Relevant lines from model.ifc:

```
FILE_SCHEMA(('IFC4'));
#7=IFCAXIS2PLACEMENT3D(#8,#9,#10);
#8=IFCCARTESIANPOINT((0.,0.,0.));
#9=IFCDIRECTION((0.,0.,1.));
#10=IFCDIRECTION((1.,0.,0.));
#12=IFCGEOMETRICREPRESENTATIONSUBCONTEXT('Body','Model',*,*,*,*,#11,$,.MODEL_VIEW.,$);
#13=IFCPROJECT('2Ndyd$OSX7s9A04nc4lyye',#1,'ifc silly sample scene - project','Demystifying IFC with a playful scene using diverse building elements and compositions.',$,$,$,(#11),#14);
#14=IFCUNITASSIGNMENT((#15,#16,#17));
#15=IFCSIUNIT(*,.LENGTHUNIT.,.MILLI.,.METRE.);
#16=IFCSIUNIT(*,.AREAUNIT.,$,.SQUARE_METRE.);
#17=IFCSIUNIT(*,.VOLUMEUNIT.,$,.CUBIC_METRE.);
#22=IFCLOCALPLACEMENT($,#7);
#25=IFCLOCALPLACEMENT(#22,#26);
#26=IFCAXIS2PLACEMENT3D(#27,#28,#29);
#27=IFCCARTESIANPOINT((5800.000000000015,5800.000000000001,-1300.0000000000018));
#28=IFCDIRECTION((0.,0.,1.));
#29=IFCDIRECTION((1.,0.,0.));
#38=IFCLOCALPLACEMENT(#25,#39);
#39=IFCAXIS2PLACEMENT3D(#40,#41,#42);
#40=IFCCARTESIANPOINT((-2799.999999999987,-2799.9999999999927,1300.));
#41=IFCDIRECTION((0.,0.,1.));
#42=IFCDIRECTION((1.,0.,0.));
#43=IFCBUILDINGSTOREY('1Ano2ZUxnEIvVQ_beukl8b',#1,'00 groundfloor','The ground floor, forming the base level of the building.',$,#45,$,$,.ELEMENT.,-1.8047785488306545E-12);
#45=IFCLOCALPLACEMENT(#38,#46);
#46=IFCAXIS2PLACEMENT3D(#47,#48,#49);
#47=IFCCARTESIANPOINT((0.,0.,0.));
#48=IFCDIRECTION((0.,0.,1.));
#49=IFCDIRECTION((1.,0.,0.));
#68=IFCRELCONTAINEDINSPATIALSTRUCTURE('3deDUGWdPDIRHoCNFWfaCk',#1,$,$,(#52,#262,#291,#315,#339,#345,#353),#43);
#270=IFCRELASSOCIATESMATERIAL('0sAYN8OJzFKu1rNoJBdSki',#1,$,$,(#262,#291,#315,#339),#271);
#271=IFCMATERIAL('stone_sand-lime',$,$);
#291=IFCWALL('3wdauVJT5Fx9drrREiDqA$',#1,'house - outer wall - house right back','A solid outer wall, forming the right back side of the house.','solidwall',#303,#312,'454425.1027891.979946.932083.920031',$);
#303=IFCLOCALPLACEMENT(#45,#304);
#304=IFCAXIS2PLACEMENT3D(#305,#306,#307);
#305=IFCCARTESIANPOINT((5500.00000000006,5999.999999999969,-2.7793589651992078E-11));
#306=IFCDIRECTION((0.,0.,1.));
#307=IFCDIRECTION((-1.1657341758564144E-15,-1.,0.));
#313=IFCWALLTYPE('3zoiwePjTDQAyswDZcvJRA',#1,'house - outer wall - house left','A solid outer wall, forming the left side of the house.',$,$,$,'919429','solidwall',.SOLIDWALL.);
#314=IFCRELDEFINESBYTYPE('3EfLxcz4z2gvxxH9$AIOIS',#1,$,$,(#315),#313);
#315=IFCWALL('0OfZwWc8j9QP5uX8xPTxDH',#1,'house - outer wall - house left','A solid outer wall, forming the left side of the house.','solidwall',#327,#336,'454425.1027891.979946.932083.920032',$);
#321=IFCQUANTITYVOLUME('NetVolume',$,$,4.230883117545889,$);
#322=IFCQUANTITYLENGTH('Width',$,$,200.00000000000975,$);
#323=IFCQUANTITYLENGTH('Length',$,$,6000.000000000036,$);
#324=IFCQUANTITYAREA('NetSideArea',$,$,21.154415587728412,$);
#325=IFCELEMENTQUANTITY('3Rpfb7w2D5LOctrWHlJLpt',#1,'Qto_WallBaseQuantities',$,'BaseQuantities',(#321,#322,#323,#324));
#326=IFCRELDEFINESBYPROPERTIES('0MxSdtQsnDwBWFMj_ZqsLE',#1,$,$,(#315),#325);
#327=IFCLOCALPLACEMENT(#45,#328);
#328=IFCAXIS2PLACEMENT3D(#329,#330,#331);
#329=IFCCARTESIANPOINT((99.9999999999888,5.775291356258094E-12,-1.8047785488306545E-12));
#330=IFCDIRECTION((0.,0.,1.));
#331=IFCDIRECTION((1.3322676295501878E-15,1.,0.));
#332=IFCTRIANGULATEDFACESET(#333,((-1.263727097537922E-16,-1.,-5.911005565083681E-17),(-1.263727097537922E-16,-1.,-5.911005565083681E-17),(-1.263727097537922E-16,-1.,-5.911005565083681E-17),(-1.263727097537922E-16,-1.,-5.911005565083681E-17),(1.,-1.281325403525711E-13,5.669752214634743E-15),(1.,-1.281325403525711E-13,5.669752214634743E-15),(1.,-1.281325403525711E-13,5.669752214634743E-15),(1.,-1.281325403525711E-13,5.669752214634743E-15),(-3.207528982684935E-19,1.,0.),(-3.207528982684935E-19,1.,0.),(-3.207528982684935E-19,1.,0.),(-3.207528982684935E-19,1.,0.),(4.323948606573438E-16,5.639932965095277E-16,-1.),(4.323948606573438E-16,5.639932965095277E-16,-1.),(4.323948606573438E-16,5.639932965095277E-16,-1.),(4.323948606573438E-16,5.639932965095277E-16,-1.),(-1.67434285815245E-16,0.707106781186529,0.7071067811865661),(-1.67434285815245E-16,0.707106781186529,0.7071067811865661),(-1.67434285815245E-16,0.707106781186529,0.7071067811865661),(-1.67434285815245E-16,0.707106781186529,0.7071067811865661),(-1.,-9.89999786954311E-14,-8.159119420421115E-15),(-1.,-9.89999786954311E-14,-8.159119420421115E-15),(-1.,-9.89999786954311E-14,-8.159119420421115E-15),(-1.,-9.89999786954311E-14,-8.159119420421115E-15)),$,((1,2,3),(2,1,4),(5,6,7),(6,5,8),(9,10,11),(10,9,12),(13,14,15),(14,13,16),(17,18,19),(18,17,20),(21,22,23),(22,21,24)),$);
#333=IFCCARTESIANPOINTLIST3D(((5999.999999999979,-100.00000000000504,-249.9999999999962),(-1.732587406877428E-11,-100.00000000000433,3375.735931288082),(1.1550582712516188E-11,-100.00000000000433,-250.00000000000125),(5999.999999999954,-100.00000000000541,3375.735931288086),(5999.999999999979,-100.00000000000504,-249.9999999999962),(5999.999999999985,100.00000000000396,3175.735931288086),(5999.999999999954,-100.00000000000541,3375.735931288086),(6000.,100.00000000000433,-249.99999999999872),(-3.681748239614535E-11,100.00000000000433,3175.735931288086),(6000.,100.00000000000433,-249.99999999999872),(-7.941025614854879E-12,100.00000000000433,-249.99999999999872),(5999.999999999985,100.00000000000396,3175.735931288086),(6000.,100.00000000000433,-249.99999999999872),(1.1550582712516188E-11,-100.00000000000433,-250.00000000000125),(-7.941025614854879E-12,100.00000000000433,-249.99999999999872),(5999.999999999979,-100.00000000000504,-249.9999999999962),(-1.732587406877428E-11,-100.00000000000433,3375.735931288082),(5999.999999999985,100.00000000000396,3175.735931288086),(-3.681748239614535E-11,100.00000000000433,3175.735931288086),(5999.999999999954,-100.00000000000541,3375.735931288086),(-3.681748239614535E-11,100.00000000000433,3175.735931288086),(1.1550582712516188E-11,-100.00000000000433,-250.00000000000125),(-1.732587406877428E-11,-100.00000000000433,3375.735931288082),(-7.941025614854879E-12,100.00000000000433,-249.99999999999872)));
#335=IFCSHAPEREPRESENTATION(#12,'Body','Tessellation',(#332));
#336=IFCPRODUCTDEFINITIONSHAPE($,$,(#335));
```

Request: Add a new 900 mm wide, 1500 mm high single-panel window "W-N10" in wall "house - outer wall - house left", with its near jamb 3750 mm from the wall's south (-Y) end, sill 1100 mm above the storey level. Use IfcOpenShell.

```python
import numpy as np
import ifcopenshell
import ifcopenshell.api.feature
import ifcopenshell.api.geometry
import ifcopenshell.api.pset
import ifcopenshell.api.root
import ifcopenshell.api.spatial
import ifcopenshell.geom
import ifcopenshell.util.element
import ifcopenshell.util.placement
import ifcopenshell.util.representation
import ifcopenshell.util.shape
import ifcopenshell.util.unit

model = ifcopenshell.open("model.ifc")
unit_scale = ifcopenshell.util.unit.calculate_unit_scale(model)
area_scale = ifcopenshell.util.unit.calculate_unit_scale(model, "AREAUNIT")
volume_scale = ifcopenshell.util.unit.calculate_unit_scale(model, "VOLUMEUNIT")
settings = ifcopenshell.geom.settings()


def volume(element):
    """Net volume in cubic metres, openings subtracted."""
    shape = ifcopenshell.geom.create_shape(settings, element)
    return ifcopenshell.util.shape.get_volume(shape.geometry)


wall = model.by_guid("0OfZwWc8j9QP5uX8xPTxDH")
storey = ifcopenshell.util.element.get_container(wall, ifc_class="IfcBuildingStorey")
context = ifcopenshell.util.representation.get_context(model, "Model", "Body", "MODEL_VIEW")
before = volume(wall)

width, height, from_end, sill = 0.9, 1.5, 3.75, 1.1  # metres

# The wall runs along its own X axis, and the end named is its -X end.
wall_shape = ifcopenshell.geom.create_shape(settings, wall)
x, y, z = ifcopenshell.util.shape.get_vertices(wall_shape.geometry).T
start = x.min() + from_end
face, thickness = float(y.min()), float(y.max() - y.min())
wall_matrix = ifcopenshell.util.placement.get_local_placement(wall.ObjectPlacement)
level = ifcopenshell.util.placement.get_local_placement(storey.ObjectPlacement)[2, 3]


def in_wall(x, y):
    """Placement at x, y metres in the wall's axes, at sill height."""
    matrix = wall_matrix.copy()
    matrix[:, 3] = wall_matrix @ np.array([x / unit_scale, y / unit_scale, 0.0, 1.0])
    matrix[2, 3] = level + sill / unit_scale
    return matrix


# Opening: a box that overshoots both wall faces by 50 mm.
opening = ifcopenshell.api.root.create_entity(model, ifc_class="IfcOpeningElement", predefined_type="OPENING")
box = ifcopenshell.api.geometry.add_wall_representation(
    model, context=context, length=width, height=height, thickness=thickness + 0.1
)
ifcopenshell.api.geometry.assign_representation(model, product=opening, representation=box)
ifcopenshell.api.geometry.edit_object_placement(model, product=opening, matrix=in_wall(start, face - 0.05), is_si=False)
ifcopenshell.api.feature.add_feature(model, feature=opening, element=wall)

window = ifcopenshell.api.root.create_entity(model, ifc_class="IfcWindow", name="W-N10", predefined_type="WINDOW")
window.OverallWidth, window.OverallHeight = width / unit_scale, height / unit_scale
window.PartitioningType = "SINGLE_PANEL"
body = ifcopenshell.api.geometry.add_window_representation(
    model,
    context=context,
    overall_width=window.OverallWidth,
    overall_height=window.OverallHeight,
    partition_type="SINGLE_PANEL",
)
ifcopenshell.api.geometry.assign_representation(model, product=window, representation=body)
ifcopenshell.api.spatial.assign_container(model, products=[window], relating_structure=storey)
ifcopenshell.api.feature.add_filling(model, opening=opening, element=window)

# Centre the window in the wall's thickness.
ifcopenshell.api.geometry.edit_object_placement(model, product=window, matrix=in_wall(start, face), is_si=False)
window_shape = ifcopenshell.geom.create_shape(settings, window)
depth = ifcopenshell.util.shape.get_vertices(window_shape.geometry)[:, 1]
offset = face + thickness / 2 - (depth.min() + depth.max()) / 2
ifcopenshell.api.geometry.edit_object_placement(model, product=window, matrix=in_wall(start, offset), is_si=False)

after = volume(wall)

# Update the wall's stored quantities.
qto = model.by_id(ifcopenshell.util.element.get_pset(wall, "Qto_WallBaseQuantities", should_inherit=False)["id"])
ifcopenshell.api.pset.edit_qto(model, qto=qto, properties={
    "NetVolume": after / volume_scale,
    "NetSideArea": after / thickness / area_scale,
})

print(f"wall volume {before:.3f} -> {after:.3f} m3")

model.write("model_v2.ifc")
```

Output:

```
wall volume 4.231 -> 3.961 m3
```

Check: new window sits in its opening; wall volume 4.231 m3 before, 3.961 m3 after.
